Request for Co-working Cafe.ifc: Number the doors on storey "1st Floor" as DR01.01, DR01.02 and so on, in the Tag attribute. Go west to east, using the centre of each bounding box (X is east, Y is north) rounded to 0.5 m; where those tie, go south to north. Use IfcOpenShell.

First a look at what the model holds.

```python
import ifcopenshell
import ifcopenshell.util.element
import ifcopenshell.util.placement

model = ifcopenshell.open("Co-working Cafe.ifc")
print(model.schema)
storey = next(s for s in model.by_type("IfcBuildingStorey") if s.Name == "1st Floor")
doors = [e for e in ifcopenshell.util.element.get_decomposition(storey) if e.is_a("IfcDoor")]
for e in sorted(doors, key=lambda e: e.id()):
    origin = ifcopenshell.util.placement.get_local_placement(e.ObjectPlacement)[:3, 3]
    print(e.id(), e.Tag, e.Name, origin.round(2) + 0.0, sep=" | ")
```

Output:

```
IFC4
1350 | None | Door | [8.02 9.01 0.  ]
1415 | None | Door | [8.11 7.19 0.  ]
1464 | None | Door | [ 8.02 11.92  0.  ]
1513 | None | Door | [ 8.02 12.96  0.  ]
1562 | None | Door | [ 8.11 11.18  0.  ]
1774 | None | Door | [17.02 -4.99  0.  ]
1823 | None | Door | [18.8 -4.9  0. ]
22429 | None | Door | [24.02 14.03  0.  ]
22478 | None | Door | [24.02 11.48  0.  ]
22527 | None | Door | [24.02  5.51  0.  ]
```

```python
import ifcopenshell
import ifcopenshell.geom
import ifcopenshell.util.element
import ifcopenshell.util.shape

model = ifcopenshell.open("Co-working Cafe.ifc")
settings = ifcopenshell.geom.settings()
settings.set("use-world-coords", True)


def centre(element):
    shape = ifcopenshell.geom.create_shape(settings, element)
    return ifcopenshell.util.shape.get_bbox_centroid(shape.geometry)


storey = next(s for s in model.by_type("IfcBuildingStorey") if s.Name == "1st Floor")
doors = [e for e in ifcopenshell.util.element.get_decomposition(storey) if e.is_a("IfcDoor")]

# Insertion points can sit at a corner or the storey origin, so sort by the geometry (in metres).
centres = {e: centre(e) for e in doors}
doors.sort(key=lambda e: (round(centres[e][0] / 0.5), centres[e][1]))

for i, e in enumerate(doors, start=1):
    number = f"DR01.{i:02d}"
    e.Tag = number
    print(e.id(), number)

model.write("Co-working Cafe_v2.ifc")
```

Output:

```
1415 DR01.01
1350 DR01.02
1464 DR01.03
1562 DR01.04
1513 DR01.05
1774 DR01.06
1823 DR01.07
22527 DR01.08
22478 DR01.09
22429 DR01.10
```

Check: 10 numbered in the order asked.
